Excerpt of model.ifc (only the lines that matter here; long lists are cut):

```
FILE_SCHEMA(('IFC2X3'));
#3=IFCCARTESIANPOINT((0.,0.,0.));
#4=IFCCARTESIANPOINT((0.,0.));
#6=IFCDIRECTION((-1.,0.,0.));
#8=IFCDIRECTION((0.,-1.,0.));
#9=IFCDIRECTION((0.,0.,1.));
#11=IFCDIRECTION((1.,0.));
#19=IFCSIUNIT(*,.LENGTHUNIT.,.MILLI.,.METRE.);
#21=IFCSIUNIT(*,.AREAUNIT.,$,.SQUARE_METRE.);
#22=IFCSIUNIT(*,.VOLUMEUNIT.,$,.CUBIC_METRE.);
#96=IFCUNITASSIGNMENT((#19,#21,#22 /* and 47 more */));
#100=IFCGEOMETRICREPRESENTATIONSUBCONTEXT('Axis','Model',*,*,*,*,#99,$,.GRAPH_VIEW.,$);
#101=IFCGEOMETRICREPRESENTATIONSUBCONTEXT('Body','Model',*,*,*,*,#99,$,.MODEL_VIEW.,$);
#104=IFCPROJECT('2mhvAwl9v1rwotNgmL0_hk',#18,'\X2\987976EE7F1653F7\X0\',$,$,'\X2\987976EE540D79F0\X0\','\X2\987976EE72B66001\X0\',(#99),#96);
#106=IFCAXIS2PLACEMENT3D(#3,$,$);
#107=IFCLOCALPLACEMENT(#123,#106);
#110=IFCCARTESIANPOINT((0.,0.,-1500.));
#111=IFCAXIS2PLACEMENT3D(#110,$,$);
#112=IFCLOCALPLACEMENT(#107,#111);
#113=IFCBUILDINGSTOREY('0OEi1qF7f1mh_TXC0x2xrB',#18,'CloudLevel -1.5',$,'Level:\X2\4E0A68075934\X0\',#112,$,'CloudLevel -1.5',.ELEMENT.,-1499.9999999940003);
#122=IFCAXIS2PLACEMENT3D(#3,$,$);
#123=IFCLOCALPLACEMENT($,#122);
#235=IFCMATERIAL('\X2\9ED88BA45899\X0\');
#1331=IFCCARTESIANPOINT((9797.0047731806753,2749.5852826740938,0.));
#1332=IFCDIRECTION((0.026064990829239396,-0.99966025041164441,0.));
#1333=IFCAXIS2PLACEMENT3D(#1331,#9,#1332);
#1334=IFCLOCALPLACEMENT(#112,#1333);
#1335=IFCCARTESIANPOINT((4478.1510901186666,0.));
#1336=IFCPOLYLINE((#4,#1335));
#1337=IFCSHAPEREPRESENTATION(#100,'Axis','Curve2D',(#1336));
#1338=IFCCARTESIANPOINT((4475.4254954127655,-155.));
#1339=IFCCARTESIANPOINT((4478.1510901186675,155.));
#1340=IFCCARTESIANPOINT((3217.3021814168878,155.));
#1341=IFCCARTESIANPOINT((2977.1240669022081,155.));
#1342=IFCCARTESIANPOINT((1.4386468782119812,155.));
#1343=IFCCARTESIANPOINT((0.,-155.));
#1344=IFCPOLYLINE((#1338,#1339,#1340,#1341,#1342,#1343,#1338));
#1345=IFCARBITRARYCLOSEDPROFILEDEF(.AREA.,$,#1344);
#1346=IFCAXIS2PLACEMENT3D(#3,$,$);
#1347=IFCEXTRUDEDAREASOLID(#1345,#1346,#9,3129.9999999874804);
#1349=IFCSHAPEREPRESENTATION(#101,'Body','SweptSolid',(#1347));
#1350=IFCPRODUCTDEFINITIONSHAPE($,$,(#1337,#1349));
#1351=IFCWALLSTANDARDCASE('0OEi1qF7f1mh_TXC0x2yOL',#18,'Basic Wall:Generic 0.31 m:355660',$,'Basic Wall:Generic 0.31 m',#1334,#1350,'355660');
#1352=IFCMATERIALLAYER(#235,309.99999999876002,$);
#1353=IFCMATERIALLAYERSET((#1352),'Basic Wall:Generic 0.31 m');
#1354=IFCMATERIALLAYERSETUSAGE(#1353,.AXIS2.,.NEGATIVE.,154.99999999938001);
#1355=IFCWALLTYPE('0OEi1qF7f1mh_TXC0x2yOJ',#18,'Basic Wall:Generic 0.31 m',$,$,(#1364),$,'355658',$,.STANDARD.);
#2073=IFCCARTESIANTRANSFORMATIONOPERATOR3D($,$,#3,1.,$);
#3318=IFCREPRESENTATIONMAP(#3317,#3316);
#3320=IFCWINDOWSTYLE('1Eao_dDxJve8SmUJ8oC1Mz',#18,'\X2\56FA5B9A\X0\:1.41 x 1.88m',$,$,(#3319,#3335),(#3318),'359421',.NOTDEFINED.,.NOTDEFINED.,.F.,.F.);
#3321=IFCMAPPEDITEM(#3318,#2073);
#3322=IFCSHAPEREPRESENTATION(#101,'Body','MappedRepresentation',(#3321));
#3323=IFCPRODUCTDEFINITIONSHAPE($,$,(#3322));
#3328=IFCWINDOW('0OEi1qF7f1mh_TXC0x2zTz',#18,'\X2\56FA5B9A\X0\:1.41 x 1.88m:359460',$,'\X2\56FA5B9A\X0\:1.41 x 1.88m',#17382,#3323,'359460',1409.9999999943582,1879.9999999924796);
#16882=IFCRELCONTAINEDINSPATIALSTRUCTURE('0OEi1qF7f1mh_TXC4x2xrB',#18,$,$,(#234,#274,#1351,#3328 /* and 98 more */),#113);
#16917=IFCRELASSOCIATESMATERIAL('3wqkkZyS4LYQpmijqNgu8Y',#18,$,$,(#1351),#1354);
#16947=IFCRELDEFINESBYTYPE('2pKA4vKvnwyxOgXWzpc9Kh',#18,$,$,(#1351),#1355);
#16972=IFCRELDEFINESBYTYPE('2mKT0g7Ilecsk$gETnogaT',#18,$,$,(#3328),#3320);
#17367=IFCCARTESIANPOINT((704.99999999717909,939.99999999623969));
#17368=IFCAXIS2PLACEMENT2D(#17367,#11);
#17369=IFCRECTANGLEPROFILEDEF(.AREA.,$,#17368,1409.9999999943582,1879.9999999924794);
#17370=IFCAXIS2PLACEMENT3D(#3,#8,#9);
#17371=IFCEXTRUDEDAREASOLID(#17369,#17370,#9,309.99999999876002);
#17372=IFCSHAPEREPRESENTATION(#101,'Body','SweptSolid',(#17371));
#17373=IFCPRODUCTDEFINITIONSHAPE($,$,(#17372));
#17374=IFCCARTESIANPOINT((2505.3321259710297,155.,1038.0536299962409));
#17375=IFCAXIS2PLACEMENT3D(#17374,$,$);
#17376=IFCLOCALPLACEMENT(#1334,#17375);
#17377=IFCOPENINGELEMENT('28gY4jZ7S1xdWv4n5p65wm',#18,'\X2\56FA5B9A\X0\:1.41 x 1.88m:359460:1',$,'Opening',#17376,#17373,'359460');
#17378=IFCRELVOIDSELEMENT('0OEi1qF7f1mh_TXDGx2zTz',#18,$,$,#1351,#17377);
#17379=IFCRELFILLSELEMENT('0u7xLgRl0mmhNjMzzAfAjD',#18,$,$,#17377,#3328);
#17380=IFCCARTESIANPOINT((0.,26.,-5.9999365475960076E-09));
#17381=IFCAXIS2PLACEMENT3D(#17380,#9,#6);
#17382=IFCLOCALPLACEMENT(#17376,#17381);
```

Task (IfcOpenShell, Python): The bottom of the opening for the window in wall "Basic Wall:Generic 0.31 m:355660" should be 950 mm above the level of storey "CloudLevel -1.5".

```python
import numpy as np
import ifcopenshell
import ifcopenshell.api.geometry
import ifcopenshell.geom
import ifcopenshell.util.element
import ifcopenshell.util.placement
import ifcopenshell.util.shape
import ifcopenshell.util.unit

model = ifcopenshell.open("model.ifc")
unit_scale = ifcopenshell.util.unit.calculate_unit_scale(model)

window = model.by_guid("0OEi1qF7f1mh_TXC0x2zTz")
opening = window.FillsVoids[0].RelatingOpeningElement
storey = ifcopenshell.util.element.get_container(window, ifc_class="IfcBuildingStorey")
level = ifcopenshell.util.placement.get_local_placement(storey.ObjectPlacement)[2, 3]

# The opening's origin need not be at the sill, so measure its lowest point.
shape = ifcopenshell.geom.create_shape(ifcopenshell.geom.settings(), opening)
bottom = ifcopenshell.util.shape.get_shape_bottom_elevation(shape, shape.geometry) / unit_scale
dz = level + 0.95 / unit_scale - bottom

shift = np.array([0.0, 0.0, dz])
# The window is placed relative to its opening, so it follows when the opening moves.
matrix = ifcopenshell.util.placement.get_local_placement(opening.ObjectPlacement)
matrix[:3, 3] += shift
ifcopenshell.api.geometry.edit_object_placement(
    model, product=opening, matrix=matrix, is_si=False, should_transform_children=True
)

print(f"moved by {dz * unit_scale:+.3f} m")

model.write("model_updated.ifc")
```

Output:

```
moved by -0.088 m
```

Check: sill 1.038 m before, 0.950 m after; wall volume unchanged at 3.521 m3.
